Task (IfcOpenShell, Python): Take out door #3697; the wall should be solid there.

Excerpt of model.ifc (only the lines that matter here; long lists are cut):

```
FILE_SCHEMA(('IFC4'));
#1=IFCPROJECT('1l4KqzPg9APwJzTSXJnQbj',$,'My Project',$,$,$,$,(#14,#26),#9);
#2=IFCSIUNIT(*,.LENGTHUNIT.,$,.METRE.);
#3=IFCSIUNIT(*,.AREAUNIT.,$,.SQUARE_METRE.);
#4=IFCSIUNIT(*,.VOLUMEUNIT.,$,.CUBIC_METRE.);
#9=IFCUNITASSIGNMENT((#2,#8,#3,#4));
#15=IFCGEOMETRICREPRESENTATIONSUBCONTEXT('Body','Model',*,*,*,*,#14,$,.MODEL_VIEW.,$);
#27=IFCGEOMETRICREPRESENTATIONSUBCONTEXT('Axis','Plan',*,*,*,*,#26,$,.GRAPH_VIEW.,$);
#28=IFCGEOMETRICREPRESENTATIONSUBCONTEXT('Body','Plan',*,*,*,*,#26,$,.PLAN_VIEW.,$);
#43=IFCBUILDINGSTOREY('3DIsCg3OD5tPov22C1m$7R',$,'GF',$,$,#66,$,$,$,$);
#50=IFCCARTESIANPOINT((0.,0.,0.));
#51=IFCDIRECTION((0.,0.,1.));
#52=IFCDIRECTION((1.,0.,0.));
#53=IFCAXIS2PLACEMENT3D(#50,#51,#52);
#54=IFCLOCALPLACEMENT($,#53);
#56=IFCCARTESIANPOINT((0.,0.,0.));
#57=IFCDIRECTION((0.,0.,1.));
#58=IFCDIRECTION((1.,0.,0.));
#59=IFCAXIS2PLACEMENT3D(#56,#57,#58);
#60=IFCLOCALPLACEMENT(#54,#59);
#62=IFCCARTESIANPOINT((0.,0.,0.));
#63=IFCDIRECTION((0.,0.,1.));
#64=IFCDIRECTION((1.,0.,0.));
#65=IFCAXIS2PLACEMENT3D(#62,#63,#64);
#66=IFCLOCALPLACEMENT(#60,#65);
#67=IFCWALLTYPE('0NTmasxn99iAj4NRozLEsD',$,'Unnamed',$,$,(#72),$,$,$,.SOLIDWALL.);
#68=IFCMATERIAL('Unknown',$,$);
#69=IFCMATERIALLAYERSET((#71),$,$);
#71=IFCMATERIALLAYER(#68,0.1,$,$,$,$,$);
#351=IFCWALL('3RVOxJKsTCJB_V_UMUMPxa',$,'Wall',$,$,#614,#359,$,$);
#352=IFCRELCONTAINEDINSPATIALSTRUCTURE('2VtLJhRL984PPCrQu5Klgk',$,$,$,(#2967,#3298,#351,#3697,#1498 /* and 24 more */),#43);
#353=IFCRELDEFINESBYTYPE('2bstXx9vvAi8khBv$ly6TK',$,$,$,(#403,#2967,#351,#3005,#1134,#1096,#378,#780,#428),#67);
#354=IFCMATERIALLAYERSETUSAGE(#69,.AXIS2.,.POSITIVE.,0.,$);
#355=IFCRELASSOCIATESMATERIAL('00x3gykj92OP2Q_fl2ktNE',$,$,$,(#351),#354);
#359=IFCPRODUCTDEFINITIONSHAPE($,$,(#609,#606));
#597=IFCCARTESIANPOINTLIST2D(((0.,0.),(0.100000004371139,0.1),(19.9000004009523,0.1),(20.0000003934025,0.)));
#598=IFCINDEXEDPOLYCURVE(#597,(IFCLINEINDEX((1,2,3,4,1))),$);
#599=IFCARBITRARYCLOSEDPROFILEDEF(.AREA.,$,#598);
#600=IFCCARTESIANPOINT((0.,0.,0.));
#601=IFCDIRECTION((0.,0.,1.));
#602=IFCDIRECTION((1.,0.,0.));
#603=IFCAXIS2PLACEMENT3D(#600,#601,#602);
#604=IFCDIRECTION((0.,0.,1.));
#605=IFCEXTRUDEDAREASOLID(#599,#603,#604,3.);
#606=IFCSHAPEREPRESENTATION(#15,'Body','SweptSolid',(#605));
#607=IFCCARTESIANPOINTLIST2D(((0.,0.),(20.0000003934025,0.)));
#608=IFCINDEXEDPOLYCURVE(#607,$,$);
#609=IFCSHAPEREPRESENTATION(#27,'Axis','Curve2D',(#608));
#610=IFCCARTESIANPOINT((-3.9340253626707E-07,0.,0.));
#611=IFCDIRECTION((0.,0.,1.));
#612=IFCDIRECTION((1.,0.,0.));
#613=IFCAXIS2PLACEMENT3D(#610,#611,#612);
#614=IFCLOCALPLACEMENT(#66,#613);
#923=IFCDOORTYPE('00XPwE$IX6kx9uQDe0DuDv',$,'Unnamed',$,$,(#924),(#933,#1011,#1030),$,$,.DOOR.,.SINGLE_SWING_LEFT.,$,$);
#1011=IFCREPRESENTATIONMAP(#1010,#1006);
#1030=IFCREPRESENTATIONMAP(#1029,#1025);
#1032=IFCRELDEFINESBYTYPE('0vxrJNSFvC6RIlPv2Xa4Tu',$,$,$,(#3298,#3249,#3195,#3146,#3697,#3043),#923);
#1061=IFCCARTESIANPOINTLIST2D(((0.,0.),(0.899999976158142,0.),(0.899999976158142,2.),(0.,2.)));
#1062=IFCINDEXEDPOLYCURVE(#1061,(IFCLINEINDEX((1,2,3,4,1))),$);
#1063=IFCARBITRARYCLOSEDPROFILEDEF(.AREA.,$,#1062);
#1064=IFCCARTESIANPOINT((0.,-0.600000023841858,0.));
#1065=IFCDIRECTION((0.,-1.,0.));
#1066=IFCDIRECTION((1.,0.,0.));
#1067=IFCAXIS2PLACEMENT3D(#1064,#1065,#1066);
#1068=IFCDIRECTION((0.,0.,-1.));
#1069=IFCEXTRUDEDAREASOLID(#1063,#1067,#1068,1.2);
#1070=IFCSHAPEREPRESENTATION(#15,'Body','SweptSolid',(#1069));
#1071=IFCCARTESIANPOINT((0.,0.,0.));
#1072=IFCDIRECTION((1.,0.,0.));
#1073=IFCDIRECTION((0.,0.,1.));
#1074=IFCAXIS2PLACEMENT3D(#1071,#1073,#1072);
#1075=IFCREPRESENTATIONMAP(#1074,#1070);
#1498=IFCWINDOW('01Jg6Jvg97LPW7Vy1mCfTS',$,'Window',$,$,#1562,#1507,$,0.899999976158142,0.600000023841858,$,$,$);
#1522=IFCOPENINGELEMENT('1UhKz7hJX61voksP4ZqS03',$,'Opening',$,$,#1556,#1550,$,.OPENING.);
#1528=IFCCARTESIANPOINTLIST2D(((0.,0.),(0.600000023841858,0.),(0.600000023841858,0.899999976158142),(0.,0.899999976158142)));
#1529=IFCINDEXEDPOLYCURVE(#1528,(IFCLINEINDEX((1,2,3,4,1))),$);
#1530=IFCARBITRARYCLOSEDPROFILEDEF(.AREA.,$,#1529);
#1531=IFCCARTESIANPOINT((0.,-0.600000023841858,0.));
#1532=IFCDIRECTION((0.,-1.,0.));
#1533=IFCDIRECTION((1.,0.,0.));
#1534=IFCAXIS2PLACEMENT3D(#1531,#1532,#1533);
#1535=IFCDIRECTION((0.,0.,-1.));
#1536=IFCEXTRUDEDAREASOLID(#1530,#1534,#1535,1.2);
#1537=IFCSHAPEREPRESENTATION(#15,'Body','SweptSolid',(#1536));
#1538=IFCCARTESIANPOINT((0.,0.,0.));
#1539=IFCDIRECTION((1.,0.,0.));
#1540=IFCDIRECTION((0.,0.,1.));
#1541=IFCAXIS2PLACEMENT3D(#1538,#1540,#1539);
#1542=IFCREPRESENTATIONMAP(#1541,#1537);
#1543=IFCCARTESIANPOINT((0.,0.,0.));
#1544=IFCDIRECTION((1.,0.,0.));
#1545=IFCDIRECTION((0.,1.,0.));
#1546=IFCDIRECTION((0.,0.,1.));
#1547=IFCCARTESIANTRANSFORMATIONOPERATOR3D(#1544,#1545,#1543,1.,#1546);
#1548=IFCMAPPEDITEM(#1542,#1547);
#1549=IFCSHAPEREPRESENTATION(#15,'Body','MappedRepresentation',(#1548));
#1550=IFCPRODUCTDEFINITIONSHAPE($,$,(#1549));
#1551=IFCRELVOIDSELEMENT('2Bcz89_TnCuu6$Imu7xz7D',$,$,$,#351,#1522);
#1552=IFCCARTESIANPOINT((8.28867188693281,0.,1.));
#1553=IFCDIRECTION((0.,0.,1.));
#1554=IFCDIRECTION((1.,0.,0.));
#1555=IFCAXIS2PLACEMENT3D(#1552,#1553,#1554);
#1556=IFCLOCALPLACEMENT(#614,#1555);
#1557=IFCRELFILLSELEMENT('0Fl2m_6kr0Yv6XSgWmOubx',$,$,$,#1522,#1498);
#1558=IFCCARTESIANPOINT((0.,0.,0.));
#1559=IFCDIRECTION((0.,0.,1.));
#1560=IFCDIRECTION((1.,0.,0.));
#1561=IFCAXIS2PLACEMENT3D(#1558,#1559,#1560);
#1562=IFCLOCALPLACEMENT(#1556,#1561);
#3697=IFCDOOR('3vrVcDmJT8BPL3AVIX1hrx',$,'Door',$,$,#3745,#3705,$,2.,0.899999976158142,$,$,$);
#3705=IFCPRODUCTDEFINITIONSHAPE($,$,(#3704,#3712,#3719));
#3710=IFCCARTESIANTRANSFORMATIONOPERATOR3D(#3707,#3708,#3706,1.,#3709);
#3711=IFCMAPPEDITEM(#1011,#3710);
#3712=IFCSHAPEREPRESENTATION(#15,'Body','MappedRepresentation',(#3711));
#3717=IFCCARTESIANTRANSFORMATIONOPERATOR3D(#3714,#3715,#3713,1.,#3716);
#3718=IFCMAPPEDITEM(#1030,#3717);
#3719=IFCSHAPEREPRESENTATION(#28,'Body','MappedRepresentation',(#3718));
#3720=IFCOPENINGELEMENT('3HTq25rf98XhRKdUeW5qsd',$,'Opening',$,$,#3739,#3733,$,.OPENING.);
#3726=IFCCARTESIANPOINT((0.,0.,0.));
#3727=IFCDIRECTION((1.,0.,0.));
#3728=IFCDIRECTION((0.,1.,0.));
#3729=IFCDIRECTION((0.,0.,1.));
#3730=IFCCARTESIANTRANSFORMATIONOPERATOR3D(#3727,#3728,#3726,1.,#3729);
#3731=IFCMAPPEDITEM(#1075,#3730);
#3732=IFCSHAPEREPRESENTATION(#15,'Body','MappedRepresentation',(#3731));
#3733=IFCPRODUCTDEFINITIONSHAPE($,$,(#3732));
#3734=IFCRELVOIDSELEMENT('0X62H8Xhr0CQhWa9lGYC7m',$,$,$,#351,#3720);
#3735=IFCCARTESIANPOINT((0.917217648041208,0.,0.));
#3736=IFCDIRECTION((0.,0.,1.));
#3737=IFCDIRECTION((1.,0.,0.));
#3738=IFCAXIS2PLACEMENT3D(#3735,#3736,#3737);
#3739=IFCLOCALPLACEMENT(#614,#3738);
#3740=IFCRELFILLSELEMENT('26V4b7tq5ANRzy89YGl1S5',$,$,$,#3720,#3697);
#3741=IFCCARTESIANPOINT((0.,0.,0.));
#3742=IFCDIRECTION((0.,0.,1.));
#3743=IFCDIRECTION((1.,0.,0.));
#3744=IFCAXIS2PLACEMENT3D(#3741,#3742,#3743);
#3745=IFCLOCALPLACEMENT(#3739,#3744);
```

```python
import ifcopenshell
import ifcopenshell.api.feature
import ifcopenshell.api.root
import ifcopenshell.geom
import ifcopenshell.util.shape

model = ifcopenshell.open("model.ifc")
settings = ifcopenshell.geom.settings()


def volume(element):
    """Net volume in cubic metres, openings subtracted."""
    shape = ifcopenshell.geom.create_shape(settings, element)
    return ifcopenshell.util.shape.get_volume(shape.geometry)


door = model.by_guid("3vrVcDmJT8BPL3AVIX1hrx")
opening = door.FillsVoids[0].RelatingOpeningElement
wall = opening.VoidsElements[0].RelatingBuildingElement
before = volume(wall)

ifcopenshell.api.root.remove_product(model, product=door)
ifcopenshell.api.feature.remove_feature(model, feature=opening)

after = volume(wall)

print(f"wall volume {before:.3f} -> {after:.3f} m3")

model.write("model_v2.ifc")
```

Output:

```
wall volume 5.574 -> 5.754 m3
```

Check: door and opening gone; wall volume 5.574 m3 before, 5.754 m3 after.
